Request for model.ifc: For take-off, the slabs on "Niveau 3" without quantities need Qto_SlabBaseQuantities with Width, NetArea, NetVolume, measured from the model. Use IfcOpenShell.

First a look at what the model holds.

```python
import ifcopenshell
import ifcopenshell.util.element
import ifcopenshell.util.unit

model = ifcopenshell.open("model.ifc")
print(model.schema)
for unit_type in ("LENGTHUNIT", "AREAUNIT", "VOLUMEUNIT"):
    print(unit_type, ifcopenshell.util.unit.calculate_unit_scale(model, unit_type))
storey = next(s for s in model.by_type("IfcBuildingStorey") if s.Name == "Niveau 3")
slabs = [e for e in ifcopenshell.util.element.get_decomposition(storey) if e.is_a("IfcSlab")]
for e in sorted(slabs, key=lambda e: e.id()):
    print(e.id(), e.is_a(), e.Name, list(ifcopenshell.util.element.get_psets(e, qtos_only=True)), sep=" | ")
```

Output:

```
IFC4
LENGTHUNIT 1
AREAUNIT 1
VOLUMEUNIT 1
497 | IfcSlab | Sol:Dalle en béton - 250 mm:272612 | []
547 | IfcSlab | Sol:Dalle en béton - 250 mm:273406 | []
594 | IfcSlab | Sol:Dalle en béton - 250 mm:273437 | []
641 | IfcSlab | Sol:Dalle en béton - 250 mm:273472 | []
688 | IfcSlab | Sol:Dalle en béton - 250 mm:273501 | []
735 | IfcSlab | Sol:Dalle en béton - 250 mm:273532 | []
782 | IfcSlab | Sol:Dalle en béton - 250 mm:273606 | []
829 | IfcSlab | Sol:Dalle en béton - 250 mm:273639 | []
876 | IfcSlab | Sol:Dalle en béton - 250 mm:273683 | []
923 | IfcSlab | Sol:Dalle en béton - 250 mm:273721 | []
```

```python
import ifcopenshell
import ifcopenshell.api.pset
import ifcopenshell.geom
import ifcopenshell.util.element
import ifcopenshell.util.shape
import ifcopenshell.util.unit

model = ifcopenshell.open("model.ifc")
unit_scale = ifcopenshell.util.unit.calculate_unit_scale(model)
area_scale = ifcopenshell.util.unit.calculate_unit_scale(model, "AREAUNIT")
volume_scale = ifcopenshell.util.unit.calculate_unit_scale(model, "VOLUMEUNIT")
settings = ifcopenshell.geom.settings()

storey = next(s for s in model.by_type("IfcBuildingStorey") if s.Name == "Niveau 3")
slabs = [e for e in ifcopenshell.util.element.get_decomposition(storey) if e.is_a("IfcSlab")]

for e in sorted(slabs, key=lambda e: e.id()):
    if ifcopenshell.util.element.get_psets(e, qtos_only=True, should_inherit=False):
        continue
    # Geometry comes back in metres, in the element's own axes.
    shape = ifcopenshell.geom.create_shape(settings, e)
    values = {
        "Width": ifcopenshell.util.shape.get_z(shape.geometry) / unit_scale,
        "NetArea": ifcopenshell.util.shape.get_footprint_area(shape.geometry) / area_scale,
        "NetVolume": ifcopenshell.util.shape.get_volume(shape.geometry) / volume_scale,
    }
    qto = ifcopenshell.api.pset.add_qto(model, product=e, name="Qto_SlabBaseQuantities")
    ifcopenshell.api.pset.edit_qto(model, qto=qto, properties=values)
    print(e.id(), {k: round(v, 3) for k, v in values.items()})

model.write("model_rev.ifc")
```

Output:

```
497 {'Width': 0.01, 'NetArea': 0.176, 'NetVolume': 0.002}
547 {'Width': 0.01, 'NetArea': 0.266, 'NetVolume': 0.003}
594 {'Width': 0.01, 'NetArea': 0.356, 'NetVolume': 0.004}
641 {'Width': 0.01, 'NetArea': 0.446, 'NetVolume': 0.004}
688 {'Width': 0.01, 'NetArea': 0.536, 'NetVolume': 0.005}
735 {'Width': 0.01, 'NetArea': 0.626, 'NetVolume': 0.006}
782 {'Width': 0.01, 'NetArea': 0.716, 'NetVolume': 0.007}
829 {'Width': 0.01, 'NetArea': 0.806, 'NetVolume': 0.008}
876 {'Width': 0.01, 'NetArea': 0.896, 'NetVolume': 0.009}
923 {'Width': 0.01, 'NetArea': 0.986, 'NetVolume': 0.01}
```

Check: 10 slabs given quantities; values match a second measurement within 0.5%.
